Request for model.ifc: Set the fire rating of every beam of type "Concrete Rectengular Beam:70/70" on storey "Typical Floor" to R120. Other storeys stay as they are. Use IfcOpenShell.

First a look at what the model holds.

```python
import ifcopenshell
import ifcopenshell.util.element

model = ifcopenshell.open("model.ifc")
print(model.schema)
storey = next(s for s in model.by_type("IfcBuildingStorey") if s.Name == "Typical Floor")
beams = [e for e in ifcopenshell.util.element.get_decomposition(storey) if e.is_a("IfcBeam")]
seen = {}
for e in beams:
    element_type = ifcopenshell.util.element.get_type(e)
    key = (element_type.Name if element_type != e and element_type else None, ifcopenshell.util.element.get_pset(e, "Pset_BeamCommon", "FireRating"))
    seen[key] = seen.get(key, 0) + 1
for (name, value), count in sorted(seen.items(), key=str):
    print(count, "x", name, "|", value)
```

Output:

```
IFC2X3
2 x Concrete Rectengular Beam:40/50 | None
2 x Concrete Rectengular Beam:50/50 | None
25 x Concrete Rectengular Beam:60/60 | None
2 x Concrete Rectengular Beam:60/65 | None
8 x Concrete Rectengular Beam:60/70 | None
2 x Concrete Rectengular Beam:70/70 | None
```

```python
import ifcopenshell
import ifcopenshell.api.pset
import ifcopenshell.util.element

model = ifcopenshell.open("model.ifc")

storey = next(s for s in model.by_type("IfcBuildingStorey") if s.Name == "Typical Floor")
beams = [e for e in ifcopenshell.util.element.get_decomposition(storey) if e.is_a("IfcBeam")]

count = 0
for e in beams:
    element_type = ifcopenshell.util.element.get_type(e)
    if element_type in (None, e) or element_type.Name != "Concrete Rectengular Beam:70/70":
        continue
    # add_pset returns the element's existing set when there is one.
    pset = ifcopenshell.api.pset.add_pset(model, product=e, name="Pset_BeamCommon")
    ifcopenshell.api.pset.edit_pset(model, pset=pset, properties={"FireRating": "R120"})
    count += 1

print(count, "beams updated")

model.write("model_edited.ifc")
```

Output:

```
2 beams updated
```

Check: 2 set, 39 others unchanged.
